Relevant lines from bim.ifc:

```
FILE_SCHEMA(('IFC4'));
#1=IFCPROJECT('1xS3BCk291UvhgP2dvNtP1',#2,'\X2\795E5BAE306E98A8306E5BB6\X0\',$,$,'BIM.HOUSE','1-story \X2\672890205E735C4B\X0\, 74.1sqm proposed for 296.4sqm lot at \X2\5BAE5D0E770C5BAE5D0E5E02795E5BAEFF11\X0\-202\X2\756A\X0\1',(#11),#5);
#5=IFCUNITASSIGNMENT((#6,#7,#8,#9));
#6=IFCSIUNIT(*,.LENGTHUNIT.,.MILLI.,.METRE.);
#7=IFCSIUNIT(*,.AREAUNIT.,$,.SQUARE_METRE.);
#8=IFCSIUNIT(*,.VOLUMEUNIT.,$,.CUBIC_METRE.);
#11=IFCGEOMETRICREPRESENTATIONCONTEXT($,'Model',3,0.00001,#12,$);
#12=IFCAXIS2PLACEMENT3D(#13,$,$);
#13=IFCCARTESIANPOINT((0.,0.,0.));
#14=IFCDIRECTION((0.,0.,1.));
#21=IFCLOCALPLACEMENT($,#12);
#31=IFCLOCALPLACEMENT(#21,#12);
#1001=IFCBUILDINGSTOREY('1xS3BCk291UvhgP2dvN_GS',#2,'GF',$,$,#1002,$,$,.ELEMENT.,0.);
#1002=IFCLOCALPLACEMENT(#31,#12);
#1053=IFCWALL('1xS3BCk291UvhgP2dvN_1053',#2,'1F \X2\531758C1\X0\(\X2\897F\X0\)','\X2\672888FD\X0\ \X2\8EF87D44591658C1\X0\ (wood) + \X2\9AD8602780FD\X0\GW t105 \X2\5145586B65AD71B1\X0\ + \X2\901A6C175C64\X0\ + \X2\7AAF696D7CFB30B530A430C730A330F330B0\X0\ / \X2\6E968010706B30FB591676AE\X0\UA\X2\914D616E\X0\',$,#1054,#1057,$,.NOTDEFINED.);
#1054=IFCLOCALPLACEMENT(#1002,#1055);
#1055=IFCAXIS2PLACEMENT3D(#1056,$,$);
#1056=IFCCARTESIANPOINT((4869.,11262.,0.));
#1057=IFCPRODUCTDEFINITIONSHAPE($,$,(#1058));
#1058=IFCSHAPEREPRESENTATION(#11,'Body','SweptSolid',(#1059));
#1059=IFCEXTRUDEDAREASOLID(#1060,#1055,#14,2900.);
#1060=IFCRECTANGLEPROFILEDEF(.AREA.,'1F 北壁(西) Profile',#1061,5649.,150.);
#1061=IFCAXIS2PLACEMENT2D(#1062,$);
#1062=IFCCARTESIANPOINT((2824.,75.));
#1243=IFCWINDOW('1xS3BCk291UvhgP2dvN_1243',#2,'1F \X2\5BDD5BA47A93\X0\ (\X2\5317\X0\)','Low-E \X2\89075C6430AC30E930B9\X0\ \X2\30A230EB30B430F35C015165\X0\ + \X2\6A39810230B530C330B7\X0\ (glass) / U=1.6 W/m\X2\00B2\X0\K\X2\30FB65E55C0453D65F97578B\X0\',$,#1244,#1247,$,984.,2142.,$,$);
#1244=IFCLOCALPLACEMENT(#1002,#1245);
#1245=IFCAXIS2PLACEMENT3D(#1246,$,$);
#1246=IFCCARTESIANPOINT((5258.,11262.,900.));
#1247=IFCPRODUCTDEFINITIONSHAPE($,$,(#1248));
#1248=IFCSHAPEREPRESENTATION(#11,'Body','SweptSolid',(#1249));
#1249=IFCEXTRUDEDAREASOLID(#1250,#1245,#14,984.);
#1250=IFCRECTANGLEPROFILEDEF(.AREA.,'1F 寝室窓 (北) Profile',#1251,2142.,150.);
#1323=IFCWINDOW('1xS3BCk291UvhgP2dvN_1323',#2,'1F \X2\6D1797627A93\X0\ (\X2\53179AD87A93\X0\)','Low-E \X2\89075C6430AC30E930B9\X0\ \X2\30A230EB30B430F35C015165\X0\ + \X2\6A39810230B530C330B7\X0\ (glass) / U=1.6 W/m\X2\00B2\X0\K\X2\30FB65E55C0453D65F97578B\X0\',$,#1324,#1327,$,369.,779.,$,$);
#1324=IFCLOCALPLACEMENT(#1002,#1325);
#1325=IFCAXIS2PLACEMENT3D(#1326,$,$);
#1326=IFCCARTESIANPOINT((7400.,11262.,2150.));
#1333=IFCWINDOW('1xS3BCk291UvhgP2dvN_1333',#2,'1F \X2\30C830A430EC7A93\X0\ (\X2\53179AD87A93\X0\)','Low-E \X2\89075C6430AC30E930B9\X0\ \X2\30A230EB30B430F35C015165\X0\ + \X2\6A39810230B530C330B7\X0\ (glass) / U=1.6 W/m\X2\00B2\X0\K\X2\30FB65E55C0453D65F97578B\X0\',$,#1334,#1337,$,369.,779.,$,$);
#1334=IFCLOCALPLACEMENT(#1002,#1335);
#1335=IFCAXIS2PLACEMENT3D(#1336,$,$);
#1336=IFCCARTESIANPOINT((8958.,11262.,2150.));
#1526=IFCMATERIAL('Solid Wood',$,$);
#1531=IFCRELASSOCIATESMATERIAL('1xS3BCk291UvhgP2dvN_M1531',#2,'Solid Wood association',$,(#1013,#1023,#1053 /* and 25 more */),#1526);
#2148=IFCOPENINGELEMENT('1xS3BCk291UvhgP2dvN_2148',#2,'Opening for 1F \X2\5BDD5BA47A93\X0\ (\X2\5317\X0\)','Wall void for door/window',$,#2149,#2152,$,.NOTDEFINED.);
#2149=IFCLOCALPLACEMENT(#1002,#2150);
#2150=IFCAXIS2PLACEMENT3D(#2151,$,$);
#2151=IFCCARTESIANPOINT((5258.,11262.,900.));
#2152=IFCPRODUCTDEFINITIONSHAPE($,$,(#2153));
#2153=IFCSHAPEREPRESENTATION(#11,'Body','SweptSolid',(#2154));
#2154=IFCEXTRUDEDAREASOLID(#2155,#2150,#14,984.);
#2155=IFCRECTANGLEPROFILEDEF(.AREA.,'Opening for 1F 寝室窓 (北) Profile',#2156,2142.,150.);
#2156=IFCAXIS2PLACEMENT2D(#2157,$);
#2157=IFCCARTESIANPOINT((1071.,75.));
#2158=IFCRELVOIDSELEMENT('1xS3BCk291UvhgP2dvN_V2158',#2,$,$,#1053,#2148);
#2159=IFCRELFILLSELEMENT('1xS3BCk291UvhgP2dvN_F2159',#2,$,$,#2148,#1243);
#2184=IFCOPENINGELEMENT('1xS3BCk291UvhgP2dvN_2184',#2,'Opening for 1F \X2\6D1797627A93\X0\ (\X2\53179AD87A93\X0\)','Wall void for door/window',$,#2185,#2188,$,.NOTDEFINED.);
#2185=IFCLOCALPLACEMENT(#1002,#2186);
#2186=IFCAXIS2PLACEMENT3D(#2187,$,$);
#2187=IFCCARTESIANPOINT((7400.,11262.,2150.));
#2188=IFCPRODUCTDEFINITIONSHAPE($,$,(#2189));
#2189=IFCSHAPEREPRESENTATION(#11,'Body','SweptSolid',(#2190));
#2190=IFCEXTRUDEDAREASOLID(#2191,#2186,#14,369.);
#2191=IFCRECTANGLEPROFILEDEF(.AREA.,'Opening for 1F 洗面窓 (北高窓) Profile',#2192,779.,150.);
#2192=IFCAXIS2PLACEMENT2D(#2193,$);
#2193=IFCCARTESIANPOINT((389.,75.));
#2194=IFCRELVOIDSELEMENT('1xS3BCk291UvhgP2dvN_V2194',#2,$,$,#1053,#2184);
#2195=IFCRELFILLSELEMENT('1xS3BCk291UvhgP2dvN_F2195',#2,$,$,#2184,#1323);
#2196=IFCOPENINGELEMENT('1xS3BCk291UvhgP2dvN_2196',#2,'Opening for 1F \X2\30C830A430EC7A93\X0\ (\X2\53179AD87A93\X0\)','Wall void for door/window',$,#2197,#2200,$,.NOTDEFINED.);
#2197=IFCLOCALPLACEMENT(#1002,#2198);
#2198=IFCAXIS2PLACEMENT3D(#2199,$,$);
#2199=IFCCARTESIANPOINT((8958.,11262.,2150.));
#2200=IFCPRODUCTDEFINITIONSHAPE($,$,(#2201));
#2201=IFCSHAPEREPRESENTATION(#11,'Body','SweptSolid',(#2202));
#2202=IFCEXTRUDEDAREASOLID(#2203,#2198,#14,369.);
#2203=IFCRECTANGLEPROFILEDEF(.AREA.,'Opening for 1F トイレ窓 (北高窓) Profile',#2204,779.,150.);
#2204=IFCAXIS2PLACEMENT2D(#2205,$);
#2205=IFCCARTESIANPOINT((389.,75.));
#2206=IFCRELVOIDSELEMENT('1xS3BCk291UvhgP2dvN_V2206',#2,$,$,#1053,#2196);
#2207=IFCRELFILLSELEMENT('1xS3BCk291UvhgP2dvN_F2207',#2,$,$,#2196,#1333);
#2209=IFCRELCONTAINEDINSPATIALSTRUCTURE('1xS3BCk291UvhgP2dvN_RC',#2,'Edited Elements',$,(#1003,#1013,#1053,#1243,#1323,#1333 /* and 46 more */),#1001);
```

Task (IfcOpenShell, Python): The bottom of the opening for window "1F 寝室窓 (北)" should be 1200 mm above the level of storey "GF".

```python
import numpy as np
import ifcopenshell
import ifcopenshell.api.geometry
import ifcopenshell.geom
import ifcopenshell.util.element
import ifcopenshell.util.placement
import ifcopenshell.util.shape
import ifcopenshell.util.unit

model = ifcopenshell.open("bim.ifc")
unit_scale = ifcopenshell.util.unit.calculate_unit_scale(model)

window = model.by_guid("1xS3BCk291UvhgP2dvN_1243")
opening = window.FillsVoids[0].RelatingOpeningElement
storey = ifcopenshell.util.element.get_container(window, ifc_class="IfcBuildingStorey")
level = ifcopenshell.util.placement.get_local_placement(storey.ObjectPlacement)[2, 3]

# The opening's origin need not be at the sill, so measure its lowest point.
shape = ifcopenshell.geom.create_shape(ifcopenshell.geom.settings(), opening)
bottom = ifcopenshell.util.shape.get_shape_bottom_elevation(shape, shape.geometry) / unit_scale
dz = level + 1200.0 - bottom

shift = np.array([0.0, 0.0, dz])
# The window is not placed relative to its opening, so move both.
for product in (opening, window):
    matrix = ifcopenshell.util.placement.get_local_placement(product.ObjectPlacement)
    matrix[:3, 3] += shift
    ifcopenshell.api.geometry.edit_object_placement(model, product=product, matrix=matrix, is_si=False)

print(f"moved by {dz * unit_scale:+.3f} m")

model.write("bim_edited.ifc")
```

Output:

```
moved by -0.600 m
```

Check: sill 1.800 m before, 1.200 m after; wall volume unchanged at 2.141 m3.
